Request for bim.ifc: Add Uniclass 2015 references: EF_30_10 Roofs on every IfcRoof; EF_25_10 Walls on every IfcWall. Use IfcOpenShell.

First a look at what the model holds.

```python
import ifcopenshell

model = ifcopenshell.open("bim.ifc")
print(model.schema)
print("classifications:", [c.Name for c in model.by_type("IfcClassification")])
for ifc_class in ("IfcDoor", "IfcRoof", "IfcStair", "IfcWall", "IfcWindow"):
    print(ifc_class, len(model.by_type(ifc_class)))
```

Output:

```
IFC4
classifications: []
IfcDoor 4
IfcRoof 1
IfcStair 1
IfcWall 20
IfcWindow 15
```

```python
import ifcopenshell
import ifcopenshell.api.classification

model = ifcopenshell.open("bim.ifc")

system = ifcopenshell.api.classification.add_classification(model, classification="Uniclass 2015")

codes = {
    "IfcRoof": ("EF_30_10", "Roofs"),
    "IfcWall": ("EF_25_10", "Walls"),
}
for ifc_class, (code, name) in codes.items():
    products = model.by_type(ifc_class)
    ifcopenshell.api.classification.add_reference(
        model, products=products, classification=system, identification=code, name=name
    )
    print(code, len(products))

model.write("bim_v2.ifc")
```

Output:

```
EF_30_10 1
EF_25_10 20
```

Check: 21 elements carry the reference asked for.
